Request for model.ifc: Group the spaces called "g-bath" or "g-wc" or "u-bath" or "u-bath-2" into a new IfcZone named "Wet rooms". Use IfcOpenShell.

First a look at what the model holds.

```python
import ifcopenshell

model = ifcopenshell.open("model.ifc")
print(model.schema)
seen = {}
for space in model.by_type("IfcSpace"):
    seen[space.LongName] = seen.get(space.LongName, 0) + 1
for name, count in sorted(seen.items(), key=str):
    print(count, "x", name)
print("zones:", [z.Name for z in model.by_type("IfcZone")][:20])
```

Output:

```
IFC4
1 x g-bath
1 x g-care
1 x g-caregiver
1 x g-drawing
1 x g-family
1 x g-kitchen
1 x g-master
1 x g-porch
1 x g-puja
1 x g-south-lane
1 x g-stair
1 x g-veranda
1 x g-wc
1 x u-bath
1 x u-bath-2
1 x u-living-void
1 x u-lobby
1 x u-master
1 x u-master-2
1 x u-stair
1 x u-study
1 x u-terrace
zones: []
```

```python
import ifcopenshell
import ifcopenshell.api.group
import ifcopenshell.api.root

model = ifcopenshell.open("model.ifc")

names = {"g-bath", "g-wc", "u-bath", "u-bath-2"}
spaces = [s for s in model.by_type("IfcSpace") if s.LongName in names]

zone = ifcopenshell.api.root.create_entity(model, ifc_class="IfcZone", name="Wet rooms")
ifcopenshell.api.group.assign_group(model, products=spaces, group=zone)
print(len(spaces), "spaces in", zone.Name)

model.write("model_rev.ifc")
```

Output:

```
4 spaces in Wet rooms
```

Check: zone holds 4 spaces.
